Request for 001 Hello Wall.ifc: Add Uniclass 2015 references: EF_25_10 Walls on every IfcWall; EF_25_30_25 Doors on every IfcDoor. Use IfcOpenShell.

First a look at what the model holds.

```python
import ifcopenshell

model = ifcopenshell.open("001 Hello Wall.ifc")
print(model.schema)
print("classifications:", [c.Name for c in model.by_type("IfcClassification")])
for ifc_class in ("IfcDoor", "IfcRoof", "IfcStair", "IfcWall", "IfcWindow"):
    print(ifc_class, len(model.by_type(ifc_class)))
```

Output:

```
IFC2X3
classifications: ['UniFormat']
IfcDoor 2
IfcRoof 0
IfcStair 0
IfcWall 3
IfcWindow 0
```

```python
import ifcopenshell
import ifcopenshell.api.classification

model = ifcopenshell.open("001 Hello Wall.ifc")

# IFC2X3 requires Source and Edition and has no link from the project to the system.
system = model.create_entity("IfcClassification", Source="NBS", Edition="2015", Name="Uniclass 2015")

codes = {
    "IfcWall": ("EF_25_10", "Walls"),
    "IfcDoor": ("EF_25_30_25", "Doors"),
}
for ifc_class, (code, name) in codes.items():
    products = model.by_type(ifc_class)
    ifcopenshell.api.classification.add_reference(
        model, products=products, classification=system, identification=code, name=name
    )
    print(code, len(products))

model.write("001 Hello Wall_updated.ifc")
```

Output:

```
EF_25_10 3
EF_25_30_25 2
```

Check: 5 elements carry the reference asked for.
